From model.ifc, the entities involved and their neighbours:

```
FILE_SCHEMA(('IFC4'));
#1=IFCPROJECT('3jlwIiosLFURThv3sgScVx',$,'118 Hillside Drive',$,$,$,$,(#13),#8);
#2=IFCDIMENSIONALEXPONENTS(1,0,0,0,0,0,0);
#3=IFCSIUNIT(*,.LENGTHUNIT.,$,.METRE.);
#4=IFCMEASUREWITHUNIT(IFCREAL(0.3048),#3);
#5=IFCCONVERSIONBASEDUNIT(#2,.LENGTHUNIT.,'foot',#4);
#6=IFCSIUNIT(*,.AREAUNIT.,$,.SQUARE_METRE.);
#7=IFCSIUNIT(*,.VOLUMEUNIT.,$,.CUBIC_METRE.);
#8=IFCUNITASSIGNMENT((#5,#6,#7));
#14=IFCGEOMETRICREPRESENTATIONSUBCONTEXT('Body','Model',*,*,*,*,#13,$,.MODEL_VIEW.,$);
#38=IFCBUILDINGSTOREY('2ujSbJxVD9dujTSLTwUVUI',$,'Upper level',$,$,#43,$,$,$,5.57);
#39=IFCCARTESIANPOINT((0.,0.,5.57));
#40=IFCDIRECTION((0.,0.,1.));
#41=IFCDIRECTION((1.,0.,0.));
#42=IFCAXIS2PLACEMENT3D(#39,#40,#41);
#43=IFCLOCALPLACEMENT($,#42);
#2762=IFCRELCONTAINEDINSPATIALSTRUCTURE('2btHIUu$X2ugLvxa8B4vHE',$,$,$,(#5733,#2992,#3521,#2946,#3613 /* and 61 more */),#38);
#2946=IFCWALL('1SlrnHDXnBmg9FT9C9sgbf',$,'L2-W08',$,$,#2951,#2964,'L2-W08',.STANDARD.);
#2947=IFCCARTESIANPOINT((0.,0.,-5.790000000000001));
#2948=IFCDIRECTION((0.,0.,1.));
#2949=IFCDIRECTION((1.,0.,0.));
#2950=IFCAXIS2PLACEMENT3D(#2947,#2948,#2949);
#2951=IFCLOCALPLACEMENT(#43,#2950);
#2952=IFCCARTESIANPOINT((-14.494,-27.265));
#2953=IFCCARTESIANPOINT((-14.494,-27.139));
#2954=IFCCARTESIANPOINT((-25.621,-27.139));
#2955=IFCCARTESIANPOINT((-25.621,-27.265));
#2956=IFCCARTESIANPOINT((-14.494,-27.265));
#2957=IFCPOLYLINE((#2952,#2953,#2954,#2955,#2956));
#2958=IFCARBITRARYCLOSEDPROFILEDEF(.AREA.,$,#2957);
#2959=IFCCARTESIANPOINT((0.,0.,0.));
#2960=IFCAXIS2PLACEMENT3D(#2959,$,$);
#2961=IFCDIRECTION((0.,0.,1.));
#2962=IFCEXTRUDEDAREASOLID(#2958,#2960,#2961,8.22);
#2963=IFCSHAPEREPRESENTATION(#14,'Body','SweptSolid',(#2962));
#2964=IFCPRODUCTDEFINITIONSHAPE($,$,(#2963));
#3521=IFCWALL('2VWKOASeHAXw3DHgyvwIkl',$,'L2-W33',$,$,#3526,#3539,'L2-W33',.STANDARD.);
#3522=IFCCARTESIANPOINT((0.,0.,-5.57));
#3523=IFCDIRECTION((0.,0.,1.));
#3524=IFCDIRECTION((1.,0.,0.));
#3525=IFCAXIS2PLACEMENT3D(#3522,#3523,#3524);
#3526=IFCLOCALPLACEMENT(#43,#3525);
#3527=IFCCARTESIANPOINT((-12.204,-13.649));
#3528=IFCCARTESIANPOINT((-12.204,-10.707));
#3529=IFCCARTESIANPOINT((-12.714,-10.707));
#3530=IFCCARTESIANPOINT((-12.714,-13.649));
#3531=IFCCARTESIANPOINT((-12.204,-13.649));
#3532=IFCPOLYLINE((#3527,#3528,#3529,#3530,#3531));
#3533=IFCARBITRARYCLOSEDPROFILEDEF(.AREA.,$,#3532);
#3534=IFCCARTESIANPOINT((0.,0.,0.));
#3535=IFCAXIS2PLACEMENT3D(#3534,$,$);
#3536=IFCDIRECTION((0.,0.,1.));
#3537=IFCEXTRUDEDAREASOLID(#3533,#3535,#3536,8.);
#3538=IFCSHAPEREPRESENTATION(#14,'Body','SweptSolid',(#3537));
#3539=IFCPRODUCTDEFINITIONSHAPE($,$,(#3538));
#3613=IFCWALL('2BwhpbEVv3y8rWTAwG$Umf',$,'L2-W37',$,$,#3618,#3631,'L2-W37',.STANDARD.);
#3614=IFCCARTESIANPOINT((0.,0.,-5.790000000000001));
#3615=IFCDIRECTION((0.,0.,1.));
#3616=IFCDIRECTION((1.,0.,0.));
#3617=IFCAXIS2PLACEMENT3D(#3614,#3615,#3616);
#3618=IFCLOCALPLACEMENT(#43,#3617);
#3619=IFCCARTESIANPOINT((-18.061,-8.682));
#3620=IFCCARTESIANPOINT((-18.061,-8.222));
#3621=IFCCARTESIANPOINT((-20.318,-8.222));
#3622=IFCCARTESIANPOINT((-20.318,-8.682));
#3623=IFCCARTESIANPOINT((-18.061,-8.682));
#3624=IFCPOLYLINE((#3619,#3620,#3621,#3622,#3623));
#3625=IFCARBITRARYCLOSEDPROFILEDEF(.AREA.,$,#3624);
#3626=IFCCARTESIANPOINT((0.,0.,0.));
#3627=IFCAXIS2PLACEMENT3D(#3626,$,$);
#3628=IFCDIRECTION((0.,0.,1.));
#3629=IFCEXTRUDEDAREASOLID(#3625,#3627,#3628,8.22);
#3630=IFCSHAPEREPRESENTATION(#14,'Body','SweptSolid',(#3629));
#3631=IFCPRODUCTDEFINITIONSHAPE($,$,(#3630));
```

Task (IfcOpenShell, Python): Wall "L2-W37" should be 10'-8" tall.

```python
import ifcopenshell
import ifcopenshell.geom
import ifcopenshell.util.representation
import ifcopenshell.util.shape
import ifcopenshell.util.unit

model = ifcopenshell.open("model.ifc")
unit_scale = ifcopenshell.util.unit.calculate_unit_scale(model)
settings = ifcopenshell.geom.settings()


def volume(element):
    """Net volume in cubic metres, openings subtracted."""
    shape = ifcopenshell.geom.create_shape(settings, element)
    return ifcopenshell.util.shape.get_volume(shape.geometry)


wall = model.by_id(3613)
before = volume(wall)

body = ifcopenshell.util.representation.get_representation(wall, "Model", "Body")
solid = body.Items[0]
old_height = solid.Depth
solid.Depth = 128 * 0.0254 / unit_scale
after = volume(wall)

print(f"height {old_height:g} -> {solid.Depth:g}, volume {before:.3f} -> {after:.3f} m3")

model.write("model_rev.ifc")
```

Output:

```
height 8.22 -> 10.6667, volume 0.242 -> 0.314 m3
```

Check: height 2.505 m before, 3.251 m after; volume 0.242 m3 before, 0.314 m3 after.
